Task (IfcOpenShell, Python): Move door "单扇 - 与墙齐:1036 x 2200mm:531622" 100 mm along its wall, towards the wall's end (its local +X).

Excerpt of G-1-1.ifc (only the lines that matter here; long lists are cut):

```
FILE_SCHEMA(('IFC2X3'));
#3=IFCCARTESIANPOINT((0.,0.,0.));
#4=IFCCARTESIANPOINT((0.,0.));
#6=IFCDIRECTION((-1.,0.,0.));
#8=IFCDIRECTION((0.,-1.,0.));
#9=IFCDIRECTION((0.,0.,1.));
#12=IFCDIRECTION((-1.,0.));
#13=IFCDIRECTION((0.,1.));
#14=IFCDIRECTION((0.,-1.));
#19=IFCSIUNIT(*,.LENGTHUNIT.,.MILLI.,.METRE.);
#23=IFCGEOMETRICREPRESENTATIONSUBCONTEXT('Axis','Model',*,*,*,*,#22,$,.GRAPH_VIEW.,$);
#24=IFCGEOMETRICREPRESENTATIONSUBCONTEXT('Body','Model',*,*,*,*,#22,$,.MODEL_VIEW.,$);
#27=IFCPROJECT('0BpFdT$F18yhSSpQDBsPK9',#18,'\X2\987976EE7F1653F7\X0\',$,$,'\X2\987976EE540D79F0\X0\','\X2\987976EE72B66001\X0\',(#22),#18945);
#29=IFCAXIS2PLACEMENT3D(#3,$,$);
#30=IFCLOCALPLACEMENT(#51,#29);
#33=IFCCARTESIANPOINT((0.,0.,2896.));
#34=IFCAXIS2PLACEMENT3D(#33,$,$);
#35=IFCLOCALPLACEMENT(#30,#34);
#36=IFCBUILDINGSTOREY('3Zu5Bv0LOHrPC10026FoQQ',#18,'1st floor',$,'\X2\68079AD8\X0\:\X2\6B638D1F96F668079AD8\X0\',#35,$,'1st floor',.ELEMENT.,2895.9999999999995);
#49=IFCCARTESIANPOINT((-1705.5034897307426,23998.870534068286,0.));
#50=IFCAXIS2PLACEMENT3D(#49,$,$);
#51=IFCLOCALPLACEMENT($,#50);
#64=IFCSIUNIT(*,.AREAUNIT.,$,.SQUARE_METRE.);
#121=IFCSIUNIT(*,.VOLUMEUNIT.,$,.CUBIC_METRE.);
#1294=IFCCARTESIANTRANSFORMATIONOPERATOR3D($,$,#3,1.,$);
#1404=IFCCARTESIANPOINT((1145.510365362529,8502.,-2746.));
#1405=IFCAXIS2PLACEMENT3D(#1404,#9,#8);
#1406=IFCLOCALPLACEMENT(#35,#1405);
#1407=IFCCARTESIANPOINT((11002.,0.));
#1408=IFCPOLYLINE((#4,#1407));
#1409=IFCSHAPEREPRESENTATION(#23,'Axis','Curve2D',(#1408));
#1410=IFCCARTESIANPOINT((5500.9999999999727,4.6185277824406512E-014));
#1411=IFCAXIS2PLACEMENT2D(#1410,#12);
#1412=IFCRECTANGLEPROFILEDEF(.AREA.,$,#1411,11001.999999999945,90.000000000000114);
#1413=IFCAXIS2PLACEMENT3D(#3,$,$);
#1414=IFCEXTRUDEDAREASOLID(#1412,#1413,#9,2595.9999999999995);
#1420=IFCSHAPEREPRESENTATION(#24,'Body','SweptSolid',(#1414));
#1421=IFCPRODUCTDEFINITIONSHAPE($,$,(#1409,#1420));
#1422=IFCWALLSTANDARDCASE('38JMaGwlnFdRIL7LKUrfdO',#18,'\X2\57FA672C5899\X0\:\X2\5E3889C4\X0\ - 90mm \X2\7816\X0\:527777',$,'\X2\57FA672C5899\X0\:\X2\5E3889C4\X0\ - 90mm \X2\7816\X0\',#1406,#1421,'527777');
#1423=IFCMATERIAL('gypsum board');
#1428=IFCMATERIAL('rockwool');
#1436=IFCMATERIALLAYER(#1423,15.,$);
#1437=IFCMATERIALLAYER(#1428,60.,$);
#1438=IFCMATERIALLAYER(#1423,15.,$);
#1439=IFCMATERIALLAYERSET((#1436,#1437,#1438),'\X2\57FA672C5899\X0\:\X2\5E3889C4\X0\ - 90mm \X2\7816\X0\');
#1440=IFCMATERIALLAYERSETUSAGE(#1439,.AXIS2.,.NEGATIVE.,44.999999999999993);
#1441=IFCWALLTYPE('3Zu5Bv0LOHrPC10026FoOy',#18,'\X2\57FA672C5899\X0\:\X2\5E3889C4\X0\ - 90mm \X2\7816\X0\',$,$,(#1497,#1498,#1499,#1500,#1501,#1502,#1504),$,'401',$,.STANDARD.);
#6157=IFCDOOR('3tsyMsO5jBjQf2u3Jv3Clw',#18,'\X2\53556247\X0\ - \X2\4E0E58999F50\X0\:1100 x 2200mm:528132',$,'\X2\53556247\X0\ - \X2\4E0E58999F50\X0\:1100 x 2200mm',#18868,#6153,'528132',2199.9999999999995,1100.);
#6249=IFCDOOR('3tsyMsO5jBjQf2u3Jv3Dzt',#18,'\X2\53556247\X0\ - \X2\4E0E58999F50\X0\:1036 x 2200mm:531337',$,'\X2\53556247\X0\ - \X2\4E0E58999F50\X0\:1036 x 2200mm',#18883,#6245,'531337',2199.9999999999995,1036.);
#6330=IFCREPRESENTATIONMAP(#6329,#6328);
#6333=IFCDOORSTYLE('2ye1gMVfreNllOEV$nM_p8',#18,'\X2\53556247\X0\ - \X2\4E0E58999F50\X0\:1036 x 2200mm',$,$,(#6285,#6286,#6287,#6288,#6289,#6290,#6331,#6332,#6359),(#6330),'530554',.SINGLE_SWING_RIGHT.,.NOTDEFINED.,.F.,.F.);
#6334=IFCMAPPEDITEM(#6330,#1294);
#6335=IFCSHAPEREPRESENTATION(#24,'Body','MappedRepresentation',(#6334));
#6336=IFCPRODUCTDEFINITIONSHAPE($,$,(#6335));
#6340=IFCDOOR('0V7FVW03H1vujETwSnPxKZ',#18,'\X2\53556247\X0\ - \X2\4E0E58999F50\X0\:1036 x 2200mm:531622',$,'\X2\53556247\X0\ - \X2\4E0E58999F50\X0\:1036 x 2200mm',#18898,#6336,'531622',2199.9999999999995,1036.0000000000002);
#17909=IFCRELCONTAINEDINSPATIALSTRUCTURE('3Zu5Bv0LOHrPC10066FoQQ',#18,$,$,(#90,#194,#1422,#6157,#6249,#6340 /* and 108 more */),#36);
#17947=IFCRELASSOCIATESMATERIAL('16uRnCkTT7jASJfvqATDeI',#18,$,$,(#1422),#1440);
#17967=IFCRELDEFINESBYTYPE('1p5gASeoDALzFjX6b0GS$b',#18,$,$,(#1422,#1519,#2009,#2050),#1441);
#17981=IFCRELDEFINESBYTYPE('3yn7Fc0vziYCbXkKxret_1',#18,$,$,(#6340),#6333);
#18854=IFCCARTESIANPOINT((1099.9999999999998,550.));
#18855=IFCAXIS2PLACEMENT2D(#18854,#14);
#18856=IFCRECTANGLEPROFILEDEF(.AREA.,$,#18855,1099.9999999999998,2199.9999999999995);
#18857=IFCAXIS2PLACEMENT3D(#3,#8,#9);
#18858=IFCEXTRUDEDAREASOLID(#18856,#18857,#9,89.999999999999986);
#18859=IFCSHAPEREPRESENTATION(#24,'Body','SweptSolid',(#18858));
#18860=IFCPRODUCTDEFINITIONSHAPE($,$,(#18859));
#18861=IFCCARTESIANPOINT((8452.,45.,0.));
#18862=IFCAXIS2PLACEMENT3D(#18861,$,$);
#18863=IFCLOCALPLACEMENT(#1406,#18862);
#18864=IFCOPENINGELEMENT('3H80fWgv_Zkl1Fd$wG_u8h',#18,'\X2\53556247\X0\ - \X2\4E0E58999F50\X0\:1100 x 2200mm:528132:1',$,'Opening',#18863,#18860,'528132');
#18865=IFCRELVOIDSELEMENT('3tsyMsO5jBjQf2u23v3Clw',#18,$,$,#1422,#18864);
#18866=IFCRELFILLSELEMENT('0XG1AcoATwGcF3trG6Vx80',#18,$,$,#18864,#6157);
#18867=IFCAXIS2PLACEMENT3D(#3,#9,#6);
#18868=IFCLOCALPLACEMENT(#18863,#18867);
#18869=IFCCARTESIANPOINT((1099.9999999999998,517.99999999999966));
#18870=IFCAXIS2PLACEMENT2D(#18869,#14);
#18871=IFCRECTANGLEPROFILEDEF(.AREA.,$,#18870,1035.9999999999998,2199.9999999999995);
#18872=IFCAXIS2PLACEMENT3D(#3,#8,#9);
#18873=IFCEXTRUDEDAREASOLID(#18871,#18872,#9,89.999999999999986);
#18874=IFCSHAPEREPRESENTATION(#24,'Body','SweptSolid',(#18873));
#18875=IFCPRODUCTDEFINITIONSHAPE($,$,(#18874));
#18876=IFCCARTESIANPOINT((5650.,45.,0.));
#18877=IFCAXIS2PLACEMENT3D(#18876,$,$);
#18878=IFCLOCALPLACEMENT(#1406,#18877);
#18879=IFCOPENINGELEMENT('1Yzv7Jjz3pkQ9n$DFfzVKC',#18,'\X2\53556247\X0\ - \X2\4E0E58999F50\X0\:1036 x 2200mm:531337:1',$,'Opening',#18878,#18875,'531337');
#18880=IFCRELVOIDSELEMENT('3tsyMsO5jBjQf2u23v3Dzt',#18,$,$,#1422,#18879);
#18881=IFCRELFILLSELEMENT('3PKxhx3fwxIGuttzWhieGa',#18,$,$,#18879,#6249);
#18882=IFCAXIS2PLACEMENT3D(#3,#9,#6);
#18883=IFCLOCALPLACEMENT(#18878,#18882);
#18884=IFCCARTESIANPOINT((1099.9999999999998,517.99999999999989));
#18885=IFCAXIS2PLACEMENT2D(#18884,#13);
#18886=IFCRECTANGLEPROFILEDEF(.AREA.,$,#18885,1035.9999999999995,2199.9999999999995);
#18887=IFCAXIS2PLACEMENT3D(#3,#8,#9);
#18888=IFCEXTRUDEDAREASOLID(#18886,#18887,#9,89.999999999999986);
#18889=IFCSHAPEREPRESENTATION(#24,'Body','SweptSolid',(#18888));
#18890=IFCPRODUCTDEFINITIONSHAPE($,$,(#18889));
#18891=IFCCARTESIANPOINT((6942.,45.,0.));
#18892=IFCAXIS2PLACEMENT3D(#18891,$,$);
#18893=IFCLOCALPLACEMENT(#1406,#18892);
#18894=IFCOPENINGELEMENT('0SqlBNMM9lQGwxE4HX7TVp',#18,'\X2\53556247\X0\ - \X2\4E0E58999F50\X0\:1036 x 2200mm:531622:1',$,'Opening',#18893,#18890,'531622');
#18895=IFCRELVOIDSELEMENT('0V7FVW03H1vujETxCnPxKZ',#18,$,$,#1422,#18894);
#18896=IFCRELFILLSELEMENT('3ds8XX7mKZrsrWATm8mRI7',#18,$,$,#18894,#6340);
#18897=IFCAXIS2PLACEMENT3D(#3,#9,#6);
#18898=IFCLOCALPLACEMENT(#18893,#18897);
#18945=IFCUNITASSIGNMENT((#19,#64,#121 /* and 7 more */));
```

```python
import ifcopenshell
import ifcopenshell.api.geometry
import ifcopenshell.util.placement
import ifcopenshell.util.unit

model = ifcopenshell.open("G-1-1.ifc")
unit_scale = ifcopenshell.util.unit.calculate_unit_scale(model)

door = model.by_guid("0V7FVW03H1vujETwSnPxKZ")
opening = door.FillsVoids[0].RelatingOpeningElement
wall = opening.VoidsElements[0].RelatingBuildingElement

wall_matrix = ifcopenshell.util.placement.get_local_placement(wall.ObjectPlacement)
shift = wall_matrix[:3, 0] * 0.1 / unit_scale
before = ifcopenshell.util.placement.get_local_placement(door.ObjectPlacement)[:3, 3].copy()

# The door is placed relative to its opening, so it follows when the opening moves.
matrix = ifcopenshell.util.placement.get_local_placement(opening.ObjectPlacement)
matrix[:3, 3] += shift
ifcopenshell.api.geometry.edit_object_placement(
    model, product=opening, matrix=matrix, is_si=False, should_transform_children=True
)

after = ifcopenshell.util.placement.get_local_placement(door.ObjectPlacement)[:3, 3]
print("door moved by", (after - before).round(3) + 0.0)

model.write("G-1-1_v2.ifc")
```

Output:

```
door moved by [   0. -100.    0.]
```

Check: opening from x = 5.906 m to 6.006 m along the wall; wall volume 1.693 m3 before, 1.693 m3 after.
